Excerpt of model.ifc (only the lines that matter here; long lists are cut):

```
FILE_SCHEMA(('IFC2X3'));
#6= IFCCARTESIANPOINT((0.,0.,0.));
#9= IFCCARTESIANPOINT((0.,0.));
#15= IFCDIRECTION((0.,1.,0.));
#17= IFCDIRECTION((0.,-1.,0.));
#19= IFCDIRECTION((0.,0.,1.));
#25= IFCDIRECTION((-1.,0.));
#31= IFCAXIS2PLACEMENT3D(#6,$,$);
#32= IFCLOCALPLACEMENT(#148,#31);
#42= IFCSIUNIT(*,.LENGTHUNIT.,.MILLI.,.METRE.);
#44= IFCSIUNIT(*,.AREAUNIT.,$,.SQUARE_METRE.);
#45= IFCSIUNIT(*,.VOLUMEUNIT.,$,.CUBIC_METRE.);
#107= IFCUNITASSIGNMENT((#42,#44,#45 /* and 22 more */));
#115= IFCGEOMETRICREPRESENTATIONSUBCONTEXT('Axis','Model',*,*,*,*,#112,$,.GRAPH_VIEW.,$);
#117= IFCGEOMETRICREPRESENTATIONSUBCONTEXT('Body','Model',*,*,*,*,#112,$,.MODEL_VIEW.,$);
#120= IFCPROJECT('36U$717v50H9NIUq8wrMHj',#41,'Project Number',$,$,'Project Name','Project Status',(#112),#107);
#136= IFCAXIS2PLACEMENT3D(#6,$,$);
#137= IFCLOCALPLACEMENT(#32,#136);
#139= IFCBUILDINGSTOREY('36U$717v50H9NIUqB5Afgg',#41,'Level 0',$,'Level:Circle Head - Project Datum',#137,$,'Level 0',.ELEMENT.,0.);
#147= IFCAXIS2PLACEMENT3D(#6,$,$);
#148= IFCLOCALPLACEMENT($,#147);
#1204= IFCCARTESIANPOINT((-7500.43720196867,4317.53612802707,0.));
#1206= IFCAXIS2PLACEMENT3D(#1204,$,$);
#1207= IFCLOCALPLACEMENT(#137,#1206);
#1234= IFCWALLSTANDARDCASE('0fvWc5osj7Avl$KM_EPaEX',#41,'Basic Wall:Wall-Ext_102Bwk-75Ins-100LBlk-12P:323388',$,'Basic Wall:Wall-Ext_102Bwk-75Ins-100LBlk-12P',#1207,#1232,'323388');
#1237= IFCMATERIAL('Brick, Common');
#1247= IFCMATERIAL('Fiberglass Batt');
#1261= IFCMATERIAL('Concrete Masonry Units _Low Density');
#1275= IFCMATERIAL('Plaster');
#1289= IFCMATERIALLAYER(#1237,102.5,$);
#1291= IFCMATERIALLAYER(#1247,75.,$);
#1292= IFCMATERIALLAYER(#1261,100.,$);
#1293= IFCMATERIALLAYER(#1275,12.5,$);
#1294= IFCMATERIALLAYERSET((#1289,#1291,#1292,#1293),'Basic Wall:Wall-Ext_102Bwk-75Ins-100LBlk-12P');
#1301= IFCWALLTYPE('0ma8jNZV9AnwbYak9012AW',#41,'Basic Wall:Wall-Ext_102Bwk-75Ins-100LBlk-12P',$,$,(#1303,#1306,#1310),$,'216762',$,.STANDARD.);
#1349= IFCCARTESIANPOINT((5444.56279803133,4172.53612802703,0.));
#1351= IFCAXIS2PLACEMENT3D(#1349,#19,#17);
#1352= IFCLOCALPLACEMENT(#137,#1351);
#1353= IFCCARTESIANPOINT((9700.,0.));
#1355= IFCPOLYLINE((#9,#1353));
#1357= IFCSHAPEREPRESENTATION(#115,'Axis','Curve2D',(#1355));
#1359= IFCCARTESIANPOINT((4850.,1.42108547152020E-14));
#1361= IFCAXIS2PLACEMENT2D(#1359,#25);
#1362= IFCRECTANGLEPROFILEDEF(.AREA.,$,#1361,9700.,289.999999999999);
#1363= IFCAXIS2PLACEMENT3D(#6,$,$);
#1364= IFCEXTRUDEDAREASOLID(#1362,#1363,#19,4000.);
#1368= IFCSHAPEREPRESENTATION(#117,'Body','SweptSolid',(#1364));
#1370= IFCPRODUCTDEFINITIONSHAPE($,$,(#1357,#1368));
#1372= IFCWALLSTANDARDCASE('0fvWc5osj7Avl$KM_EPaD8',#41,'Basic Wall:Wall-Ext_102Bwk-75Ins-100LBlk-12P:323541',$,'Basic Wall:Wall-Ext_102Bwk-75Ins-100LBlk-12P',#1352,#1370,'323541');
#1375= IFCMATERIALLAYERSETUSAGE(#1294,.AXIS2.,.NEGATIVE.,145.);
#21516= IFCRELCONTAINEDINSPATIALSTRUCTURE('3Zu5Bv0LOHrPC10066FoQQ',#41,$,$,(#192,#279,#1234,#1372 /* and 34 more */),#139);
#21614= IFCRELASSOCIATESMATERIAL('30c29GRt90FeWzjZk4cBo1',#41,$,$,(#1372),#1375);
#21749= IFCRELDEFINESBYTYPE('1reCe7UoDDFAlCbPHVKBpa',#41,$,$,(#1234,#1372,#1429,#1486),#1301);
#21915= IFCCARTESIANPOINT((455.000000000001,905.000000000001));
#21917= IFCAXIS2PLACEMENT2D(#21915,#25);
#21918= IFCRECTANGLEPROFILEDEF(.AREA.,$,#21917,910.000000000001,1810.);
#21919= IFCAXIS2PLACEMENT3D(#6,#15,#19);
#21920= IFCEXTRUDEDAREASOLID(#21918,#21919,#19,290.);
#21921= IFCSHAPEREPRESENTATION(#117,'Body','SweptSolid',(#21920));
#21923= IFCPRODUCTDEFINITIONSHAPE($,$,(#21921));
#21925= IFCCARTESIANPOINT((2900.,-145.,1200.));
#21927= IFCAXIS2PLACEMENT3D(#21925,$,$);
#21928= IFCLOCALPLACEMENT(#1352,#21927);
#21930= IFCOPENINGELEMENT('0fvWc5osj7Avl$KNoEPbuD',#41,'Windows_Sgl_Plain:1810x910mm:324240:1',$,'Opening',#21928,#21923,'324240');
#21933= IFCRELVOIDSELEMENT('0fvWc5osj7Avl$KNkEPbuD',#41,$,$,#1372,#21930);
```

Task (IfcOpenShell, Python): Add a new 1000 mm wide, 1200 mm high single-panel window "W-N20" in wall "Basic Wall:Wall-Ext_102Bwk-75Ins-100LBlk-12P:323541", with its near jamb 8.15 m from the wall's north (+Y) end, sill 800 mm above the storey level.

```python
import numpy as np
import ifcopenshell
import ifcopenshell.api.feature
import ifcopenshell.api.geometry
import ifcopenshell.api.root
import ifcopenshell.api.spatial
import ifcopenshell.api.type
import ifcopenshell.geom
import ifcopenshell.util.element
import ifcopenshell.util.placement
import ifcopenshell.util.representation
import ifcopenshell.util.shape
import ifcopenshell.util.unit

model = ifcopenshell.open("model.ifc")
unit_scale = ifcopenshell.util.unit.calculate_unit_scale(model)
settings = ifcopenshell.geom.settings()


def volume(element):
    """Net volume in cubic metres, openings subtracted."""
    shape = ifcopenshell.geom.create_shape(settings, element)
    return ifcopenshell.util.shape.get_volume(shape.geometry)


wall = model.by_id(1372)
storey = ifcopenshell.util.element.get_container(wall, ifc_class="IfcBuildingStorey")
context = ifcopenshell.util.representation.get_context(model, "Model", "Body", "MODEL_VIEW")
before = volume(wall)

width, height, from_end, sill = 1, 1.2, 8.15, 0.8  # metres

# The wall runs along its own X axis, and the end named is its -X end.
wall_shape = ifcopenshell.geom.create_shape(settings, wall)
x, y, z = ifcopenshell.util.shape.get_vertices(wall_shape.geometry).T
start = x.min() + from_end
face, thickness = float(y.min()), float(y.max() - y.min())
wall_matrix = ifcopenshell.util.placement.get_local_placement(wall.ObjectPlacement)
level = ifcopenshell.util.placement.get_local_placement(storey.ObjectPlacement)[2, 3]


def in_wall(x, y):
    """Placement at x, y metres in the wall's axes, at sill height."""
    matrix = wall_matrix.copy()
    matrix[:, 3] = wall_matrix @ np.array([x / unit_scale, y / unit_scale, 0.0, 1.0])
    matrix[2, 3] = level + sill / unit_scale
    return matrix


# Opening: a box that overshoots both wall faces by 50 mm.
opening = ifcopenshell.api.root.create_entity(model, ifc_class="IfcOpeningElement")
box = ifcopenshell.api.geometry.add_wall_representation(
    model, context=context, length=width, height=height, thickness=thickness + 0.1
)
ifcopenshell.api.geometry.assign_representation(model, product=opening, representation=box)
ifcopenshell.api.geometry.edit_object_placement(model, product=opening, matrix=in_wall(start, face - 0.05), is_si=False)
ifcopenshell.api.feature.add_feature(model, feature=opening, element=wall)

window = ifcopenshell.api.root.create_entity(model, ifc_class="IfcWindow", name="W-N20")
window.OverallWidth, window.OverallHeight = width / unit_scale, height / unit_scale
body = ifcopenshell.api.geometry.add_window_representation(
    model,
    context=context,
    overall_width=window.OverallWidth,
    overall_height=window.OverallHeight,
    partition_type="SINGLE_PANEL",
)
ifcopenshell.api.geometry.assign_representation(model, product=window, representation=body)
ifcopenshell.api.spatial.assign_container(model, products=[window], relating_structure=storey)
fills = ifcopenshell.api.feature.add_filling(model, opening=opening, element=window)
fills.OwnerHistory = window.OwnerHistory  # required in IFC2X3

# IFC2X3 keeps the operation on the window style.
style = ifcopenshell.api.root.create_entity(model, ifc_class="IfcWindowStyle", name="W-N20")
style.OperationType, style.ConstructionType = "SINGLE_PANEL", "NOTDEFINED"
style.ParameterTakesPrecedence = style.Sizeable = False
ifcopenshell.api.type.assign_type(model, related_objects=[window], relating_type=style)

# Centre the window in the wall's thickness.
ifcopenshell.api.geometry.edit_object_placement(model, product=window, matrix=in_wall(start, face), is_si=False)
window_shape = ifcopenshell.geom.create_shape(settings, window)
depth = ifcopenshell.util.shape.get_vertices(window_shape.geometry)[:, 1]
offset = face + thickness / 2 - (depth.min() + depth.max()) / 2
ifcopenshell.api.geometry.edit_object_placement(model, product=window, matrix=in_wall(start, offset), is_si=False)

after = volume(wall)

print(f"wall volume {before:.3f} -> {after:.3f} m3")

model.write("model-out.ifc")
```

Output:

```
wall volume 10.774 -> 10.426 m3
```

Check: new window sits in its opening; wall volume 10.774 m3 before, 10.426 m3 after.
